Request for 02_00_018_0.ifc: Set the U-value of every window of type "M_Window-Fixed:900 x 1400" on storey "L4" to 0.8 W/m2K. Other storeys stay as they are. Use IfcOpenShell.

First a look at what the model holds.

```python
import ifcopenshell
import ifcopenshell.util.element

model = ifcopenshell.open("02_00_018_0.ifc")
print(model.schema)
storey = next(s for s in model.by_type("IfcBuildingStorey") if s.Name == "L4")
windows = [e for e in ifcopenshell.util.element.get_decomposition(storey) if e.is_a("IfcWindow")]
seen = {}
for e in windows:
    element_type = ifcopenshell.util.element.get_type(e)
    key = (element_type.Name if element_type != e and element_type else None, ifcopenshell.util.element.get_pset(e, "Pset_WindowCommon", "ThermalTransmittance"))
    seen[key] = seen.get(key, 0) + 1
for (name, value), count in sorted(seen.items(), key=str):
    print(count, "x", name, "|", value)
```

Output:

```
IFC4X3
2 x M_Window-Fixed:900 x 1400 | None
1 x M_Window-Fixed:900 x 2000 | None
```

```python
import ifcopenshell
import ifcopenshell.api.pset
import ifcopenshell.util.element

model = ifcopenshell.open("02_00_018_0.ifc")

storey = next(s for s in model.by_type("IfcBuildingStorey") if s.Name == "L4")
windows = [e for e in ifcopenshell.util.element.get_decomposition(storey) if e.is_a("IfcWindow")]

count = 0
for e in windows:
    element_type = ifcopenshell.util.element.get_type(e)
    if element_type in (None, e) or element_type.Name != "M_Window-Fixed:900 x 1400":
        continue
    # add_pset returns the element's existing set when there is one.
    pset = ifcopenshell.api.pset.add_pset(model, product=e, name="Pset_WindowCommon")
    ifcopenshell.api.pset.edit_pset(model, pset=pset, properties={"ThermalTransmittance": 0.8})
    count += 1

print(count, "windows updated")

model.write("02_00_018_0-out.ifc")
```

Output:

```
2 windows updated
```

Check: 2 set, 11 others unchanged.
